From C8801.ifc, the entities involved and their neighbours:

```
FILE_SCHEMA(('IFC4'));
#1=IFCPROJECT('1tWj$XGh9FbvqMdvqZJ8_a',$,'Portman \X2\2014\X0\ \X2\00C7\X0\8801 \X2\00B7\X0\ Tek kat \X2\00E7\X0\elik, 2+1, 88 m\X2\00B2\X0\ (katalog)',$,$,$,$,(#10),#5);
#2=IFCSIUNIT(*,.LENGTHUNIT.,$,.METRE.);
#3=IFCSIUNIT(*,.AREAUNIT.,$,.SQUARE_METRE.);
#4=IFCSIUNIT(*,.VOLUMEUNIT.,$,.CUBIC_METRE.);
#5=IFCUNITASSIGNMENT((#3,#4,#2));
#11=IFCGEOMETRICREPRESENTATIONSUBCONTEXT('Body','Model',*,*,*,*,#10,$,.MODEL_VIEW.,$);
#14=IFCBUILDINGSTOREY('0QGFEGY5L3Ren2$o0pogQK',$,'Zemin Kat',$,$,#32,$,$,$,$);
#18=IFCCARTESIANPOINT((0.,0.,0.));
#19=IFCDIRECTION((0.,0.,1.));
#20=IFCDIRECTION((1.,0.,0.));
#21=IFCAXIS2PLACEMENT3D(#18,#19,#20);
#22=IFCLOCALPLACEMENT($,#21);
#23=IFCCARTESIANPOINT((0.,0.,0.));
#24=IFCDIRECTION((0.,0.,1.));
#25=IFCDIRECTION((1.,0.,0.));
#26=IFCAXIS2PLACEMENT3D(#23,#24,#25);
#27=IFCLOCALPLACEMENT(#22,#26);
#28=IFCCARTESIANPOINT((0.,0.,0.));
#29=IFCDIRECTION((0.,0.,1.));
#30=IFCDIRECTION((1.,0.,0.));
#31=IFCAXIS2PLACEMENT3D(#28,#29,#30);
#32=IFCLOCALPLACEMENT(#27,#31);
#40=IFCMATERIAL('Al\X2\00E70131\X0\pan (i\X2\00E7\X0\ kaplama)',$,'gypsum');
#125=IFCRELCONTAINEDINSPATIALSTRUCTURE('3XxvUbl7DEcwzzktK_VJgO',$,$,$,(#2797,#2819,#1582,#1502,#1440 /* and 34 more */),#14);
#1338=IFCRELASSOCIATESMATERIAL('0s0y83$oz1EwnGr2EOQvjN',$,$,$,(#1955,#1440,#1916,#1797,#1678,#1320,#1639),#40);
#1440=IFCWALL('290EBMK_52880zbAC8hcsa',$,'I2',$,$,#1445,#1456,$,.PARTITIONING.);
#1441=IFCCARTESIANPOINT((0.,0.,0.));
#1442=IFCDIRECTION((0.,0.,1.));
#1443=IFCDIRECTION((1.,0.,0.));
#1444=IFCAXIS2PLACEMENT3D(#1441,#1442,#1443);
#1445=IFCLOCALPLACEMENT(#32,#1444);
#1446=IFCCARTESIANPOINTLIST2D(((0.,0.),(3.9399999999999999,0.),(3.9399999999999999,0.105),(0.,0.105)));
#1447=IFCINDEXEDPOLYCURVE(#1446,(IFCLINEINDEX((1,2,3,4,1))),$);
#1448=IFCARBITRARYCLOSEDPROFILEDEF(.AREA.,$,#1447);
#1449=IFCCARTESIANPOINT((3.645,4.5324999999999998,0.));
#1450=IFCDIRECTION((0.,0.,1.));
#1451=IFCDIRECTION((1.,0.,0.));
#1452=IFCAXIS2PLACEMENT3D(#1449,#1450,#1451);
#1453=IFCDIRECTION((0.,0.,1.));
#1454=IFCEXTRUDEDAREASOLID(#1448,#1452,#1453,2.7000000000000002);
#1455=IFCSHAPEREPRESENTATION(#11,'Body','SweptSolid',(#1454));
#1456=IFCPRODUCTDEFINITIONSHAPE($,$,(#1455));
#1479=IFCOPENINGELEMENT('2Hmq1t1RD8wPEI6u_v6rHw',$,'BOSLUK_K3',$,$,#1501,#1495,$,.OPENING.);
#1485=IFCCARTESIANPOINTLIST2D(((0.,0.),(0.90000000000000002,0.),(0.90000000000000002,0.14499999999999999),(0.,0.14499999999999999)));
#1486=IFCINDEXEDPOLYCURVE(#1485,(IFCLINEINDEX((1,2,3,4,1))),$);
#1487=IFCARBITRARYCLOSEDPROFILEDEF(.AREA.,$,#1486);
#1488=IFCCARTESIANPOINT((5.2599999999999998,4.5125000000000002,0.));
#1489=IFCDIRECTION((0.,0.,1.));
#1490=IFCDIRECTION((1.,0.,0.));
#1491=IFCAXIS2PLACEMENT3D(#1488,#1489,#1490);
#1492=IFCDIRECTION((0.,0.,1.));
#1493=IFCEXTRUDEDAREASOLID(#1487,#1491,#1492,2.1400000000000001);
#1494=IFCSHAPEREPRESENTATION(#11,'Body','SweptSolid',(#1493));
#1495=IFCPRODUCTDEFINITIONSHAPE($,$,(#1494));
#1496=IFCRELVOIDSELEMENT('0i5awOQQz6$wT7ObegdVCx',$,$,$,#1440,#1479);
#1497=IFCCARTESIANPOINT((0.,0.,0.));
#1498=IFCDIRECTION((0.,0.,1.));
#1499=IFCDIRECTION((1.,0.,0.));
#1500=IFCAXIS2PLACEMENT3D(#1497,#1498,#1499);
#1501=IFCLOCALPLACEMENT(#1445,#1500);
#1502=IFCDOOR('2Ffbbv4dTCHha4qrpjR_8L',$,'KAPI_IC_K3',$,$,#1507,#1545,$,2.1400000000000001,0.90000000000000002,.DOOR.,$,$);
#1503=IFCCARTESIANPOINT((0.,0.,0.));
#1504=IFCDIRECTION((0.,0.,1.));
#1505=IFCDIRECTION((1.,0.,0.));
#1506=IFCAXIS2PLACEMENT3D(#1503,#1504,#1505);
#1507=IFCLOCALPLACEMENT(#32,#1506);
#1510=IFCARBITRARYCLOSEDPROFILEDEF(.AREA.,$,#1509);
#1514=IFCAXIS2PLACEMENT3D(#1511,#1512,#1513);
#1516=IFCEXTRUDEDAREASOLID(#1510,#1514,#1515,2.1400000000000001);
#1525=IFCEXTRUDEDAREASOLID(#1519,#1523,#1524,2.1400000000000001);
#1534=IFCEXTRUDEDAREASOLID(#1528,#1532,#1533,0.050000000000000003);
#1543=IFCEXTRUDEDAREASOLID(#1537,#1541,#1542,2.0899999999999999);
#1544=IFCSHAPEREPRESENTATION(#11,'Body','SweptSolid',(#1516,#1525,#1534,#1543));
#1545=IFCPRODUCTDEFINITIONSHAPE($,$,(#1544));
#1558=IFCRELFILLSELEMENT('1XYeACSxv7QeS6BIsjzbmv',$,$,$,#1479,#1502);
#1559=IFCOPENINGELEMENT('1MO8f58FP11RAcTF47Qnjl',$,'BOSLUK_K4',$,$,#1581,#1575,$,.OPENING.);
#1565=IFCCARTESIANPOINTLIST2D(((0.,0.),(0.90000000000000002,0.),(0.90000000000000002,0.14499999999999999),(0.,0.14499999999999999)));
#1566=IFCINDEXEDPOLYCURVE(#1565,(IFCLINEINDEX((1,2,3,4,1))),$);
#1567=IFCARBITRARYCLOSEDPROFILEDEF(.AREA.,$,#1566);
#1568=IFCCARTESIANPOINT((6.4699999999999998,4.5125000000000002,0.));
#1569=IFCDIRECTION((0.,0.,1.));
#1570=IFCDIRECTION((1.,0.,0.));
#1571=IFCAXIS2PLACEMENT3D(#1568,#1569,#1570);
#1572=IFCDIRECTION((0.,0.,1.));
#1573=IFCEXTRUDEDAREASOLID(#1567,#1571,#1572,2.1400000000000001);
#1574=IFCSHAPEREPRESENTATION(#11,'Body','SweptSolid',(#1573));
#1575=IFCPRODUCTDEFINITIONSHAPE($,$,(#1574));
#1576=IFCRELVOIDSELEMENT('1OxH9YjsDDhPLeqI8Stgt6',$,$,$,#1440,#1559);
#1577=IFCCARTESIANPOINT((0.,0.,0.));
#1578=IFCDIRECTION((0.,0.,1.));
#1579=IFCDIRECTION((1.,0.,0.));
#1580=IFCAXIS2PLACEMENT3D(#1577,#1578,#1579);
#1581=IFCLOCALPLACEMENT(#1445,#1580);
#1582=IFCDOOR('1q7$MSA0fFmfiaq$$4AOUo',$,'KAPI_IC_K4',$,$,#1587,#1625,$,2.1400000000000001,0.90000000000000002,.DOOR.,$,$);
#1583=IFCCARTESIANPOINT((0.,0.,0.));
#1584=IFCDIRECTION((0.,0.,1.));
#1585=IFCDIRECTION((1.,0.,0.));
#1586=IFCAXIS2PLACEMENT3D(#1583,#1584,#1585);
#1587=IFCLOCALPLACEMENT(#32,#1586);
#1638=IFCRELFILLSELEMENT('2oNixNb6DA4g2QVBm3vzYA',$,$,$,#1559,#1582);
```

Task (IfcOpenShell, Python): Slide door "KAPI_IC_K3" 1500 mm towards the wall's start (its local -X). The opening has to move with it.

```python
import ifcopenshell
import ifcopenshell.api.geometry
import ifcopenshell.util.placement
import ifcopenshell.util.unit

model = ifcopenshell.open("C8801.ifc")
unit_scale = ifcopenshell.util.unit.calculate_unit_scale(model)

door = model.by_guid("2Ffbbv4dTCHha4qrpjR_8L")
opening = door.FillsVoids[0].RelatingOpeningElement
wall = opening.VoidsElements[0].RelatingBuildingElement

wall_matrix = ifcopenshell.util.placement.get_local_placement(wall.ObjectPlacement)
shift = wall_matrix[:3, 0] * -1.5 / unit_scale
before = ifcopenshell.util.placement.get_local_placement(door.ObjectPlacement)[:3, 3].copy()

# The door is not placed relative to its opening, so move both.
for product in (opening, door):
    matrix = ifcopenshell.util.placement.get_local_placement(product.ObjectPlacement)
    matrix[:3, 3] += shift
    ifcopenshell.api.geometry.edit_object_placement(model, product=product, matrix=matrix, is_si=False)

after = ifcopenshell.util.placement.get_local_placement(door.ObjectPlacement)[:3, 3]
print("door moved by", (after - before).round(3) + 0.0)

model.write("C8801_rev.ifc")
```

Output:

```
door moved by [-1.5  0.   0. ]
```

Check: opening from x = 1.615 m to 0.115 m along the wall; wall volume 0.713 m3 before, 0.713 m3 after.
